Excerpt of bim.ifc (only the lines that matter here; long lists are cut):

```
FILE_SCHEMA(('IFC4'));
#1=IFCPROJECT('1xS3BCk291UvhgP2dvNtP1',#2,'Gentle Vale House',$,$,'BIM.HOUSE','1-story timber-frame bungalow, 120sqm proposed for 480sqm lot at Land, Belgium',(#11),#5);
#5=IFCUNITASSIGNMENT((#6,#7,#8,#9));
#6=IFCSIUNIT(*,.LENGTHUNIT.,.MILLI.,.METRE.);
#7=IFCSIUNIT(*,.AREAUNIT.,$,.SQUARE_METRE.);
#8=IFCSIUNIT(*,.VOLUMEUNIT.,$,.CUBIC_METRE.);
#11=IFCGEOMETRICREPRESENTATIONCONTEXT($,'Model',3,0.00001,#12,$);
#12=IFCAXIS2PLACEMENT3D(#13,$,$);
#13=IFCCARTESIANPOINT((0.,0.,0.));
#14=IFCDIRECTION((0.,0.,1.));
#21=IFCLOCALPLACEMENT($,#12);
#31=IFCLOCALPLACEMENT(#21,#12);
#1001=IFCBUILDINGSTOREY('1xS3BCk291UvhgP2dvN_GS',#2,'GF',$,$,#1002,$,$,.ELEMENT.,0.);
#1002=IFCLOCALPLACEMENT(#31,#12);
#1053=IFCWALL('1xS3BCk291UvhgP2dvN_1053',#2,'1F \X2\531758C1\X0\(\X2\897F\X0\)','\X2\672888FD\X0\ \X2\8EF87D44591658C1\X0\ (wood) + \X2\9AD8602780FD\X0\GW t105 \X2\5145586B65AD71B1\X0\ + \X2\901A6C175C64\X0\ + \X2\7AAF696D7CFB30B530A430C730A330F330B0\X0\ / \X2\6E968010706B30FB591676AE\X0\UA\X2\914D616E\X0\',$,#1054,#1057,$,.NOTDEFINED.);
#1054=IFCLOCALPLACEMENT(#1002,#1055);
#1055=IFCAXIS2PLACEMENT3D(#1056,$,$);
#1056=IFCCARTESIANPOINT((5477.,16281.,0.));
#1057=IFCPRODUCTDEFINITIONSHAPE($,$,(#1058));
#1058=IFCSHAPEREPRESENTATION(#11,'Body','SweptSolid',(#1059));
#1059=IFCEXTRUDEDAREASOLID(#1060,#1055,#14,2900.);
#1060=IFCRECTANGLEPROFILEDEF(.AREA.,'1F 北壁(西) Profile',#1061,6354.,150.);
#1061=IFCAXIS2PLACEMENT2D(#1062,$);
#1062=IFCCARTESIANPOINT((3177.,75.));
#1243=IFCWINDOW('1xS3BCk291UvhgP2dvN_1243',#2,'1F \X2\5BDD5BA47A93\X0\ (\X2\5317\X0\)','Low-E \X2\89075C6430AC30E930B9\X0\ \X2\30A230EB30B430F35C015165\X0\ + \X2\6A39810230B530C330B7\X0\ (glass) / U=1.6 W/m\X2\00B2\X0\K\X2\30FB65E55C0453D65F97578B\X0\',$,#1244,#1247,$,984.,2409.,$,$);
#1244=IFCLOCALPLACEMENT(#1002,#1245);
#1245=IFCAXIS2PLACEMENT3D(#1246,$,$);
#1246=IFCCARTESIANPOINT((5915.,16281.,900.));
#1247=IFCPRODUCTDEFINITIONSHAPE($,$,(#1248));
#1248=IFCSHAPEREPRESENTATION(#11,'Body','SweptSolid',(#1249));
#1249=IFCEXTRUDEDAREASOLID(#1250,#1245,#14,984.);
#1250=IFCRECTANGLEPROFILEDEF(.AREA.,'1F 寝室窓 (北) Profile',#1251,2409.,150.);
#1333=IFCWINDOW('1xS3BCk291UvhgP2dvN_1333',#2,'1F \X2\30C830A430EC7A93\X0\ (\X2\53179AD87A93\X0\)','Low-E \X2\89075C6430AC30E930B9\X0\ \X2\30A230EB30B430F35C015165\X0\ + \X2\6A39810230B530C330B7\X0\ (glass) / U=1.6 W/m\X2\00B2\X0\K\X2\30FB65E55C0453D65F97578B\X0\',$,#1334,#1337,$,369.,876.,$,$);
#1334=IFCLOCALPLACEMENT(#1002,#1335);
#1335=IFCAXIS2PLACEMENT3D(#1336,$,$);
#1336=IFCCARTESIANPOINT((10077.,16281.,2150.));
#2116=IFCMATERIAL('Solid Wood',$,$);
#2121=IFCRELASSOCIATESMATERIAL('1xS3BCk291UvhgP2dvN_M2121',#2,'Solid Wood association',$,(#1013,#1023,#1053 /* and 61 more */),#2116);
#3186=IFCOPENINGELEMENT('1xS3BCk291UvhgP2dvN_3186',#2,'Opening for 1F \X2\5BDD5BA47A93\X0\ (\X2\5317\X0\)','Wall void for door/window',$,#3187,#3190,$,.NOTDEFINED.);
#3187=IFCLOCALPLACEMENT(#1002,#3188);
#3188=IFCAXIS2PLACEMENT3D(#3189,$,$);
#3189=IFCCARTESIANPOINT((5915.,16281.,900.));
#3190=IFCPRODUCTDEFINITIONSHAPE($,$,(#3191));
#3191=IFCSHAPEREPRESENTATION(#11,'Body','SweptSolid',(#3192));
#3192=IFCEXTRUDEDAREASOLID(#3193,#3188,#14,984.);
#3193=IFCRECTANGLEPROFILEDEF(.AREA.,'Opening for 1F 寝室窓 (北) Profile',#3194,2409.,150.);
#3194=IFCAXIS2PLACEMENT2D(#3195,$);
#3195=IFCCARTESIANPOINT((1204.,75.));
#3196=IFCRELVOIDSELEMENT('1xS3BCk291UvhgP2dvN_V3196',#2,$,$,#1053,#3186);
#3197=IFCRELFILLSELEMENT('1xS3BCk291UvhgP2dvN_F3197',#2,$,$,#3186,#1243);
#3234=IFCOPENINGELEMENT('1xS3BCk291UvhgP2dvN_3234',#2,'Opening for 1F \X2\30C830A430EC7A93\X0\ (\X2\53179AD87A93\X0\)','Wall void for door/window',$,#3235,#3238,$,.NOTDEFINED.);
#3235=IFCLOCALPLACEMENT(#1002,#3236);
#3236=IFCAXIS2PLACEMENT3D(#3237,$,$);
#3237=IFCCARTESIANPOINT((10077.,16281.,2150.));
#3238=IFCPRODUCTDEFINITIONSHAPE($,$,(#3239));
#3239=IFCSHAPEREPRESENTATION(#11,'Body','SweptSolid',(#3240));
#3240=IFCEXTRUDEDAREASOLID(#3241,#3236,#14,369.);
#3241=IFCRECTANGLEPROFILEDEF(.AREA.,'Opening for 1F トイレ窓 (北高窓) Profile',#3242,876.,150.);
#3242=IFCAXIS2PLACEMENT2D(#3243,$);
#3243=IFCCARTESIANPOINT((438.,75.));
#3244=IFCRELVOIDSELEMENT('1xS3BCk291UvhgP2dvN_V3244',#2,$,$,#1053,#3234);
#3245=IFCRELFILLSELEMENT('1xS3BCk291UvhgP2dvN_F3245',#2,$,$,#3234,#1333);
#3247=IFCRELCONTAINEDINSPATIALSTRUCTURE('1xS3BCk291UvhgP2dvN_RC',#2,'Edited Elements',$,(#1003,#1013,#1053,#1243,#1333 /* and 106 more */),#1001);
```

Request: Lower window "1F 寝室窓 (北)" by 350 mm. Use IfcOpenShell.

```python
import numpy as np
import ifcopenshell
import ifcopenshell.api.geometry
import ifcopenshell.util.placement
import ifcopenshell.util.unit

model = ifcopenshell.open("bim.ifc")
unit_scale = ifcopenshell.util.unit.calculate_unit_scale(model)

window = model.by_id(1243)
opening = window.FillsVoids[0].RelatingOpeningElement
dz = -350.0

shift = np.array([0.0, 0.0, dz])
# The window is not placed relative to its opening, so move both.
for product in (opening, window):
    matrix = ifcopenshell.util.placement.get_local_placement(product.ObjectPlacement)
    matrix[:3, 3] += shift
    ifcopenshell.api.geometry.edit_object_placement(model, product=product, matrix=matrix, is_si=False)

print(f"moved by {dz * unit_scale:+.3f} m")

model.write("bim_edited.ifc")
```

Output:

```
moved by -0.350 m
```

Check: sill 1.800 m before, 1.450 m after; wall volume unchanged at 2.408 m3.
